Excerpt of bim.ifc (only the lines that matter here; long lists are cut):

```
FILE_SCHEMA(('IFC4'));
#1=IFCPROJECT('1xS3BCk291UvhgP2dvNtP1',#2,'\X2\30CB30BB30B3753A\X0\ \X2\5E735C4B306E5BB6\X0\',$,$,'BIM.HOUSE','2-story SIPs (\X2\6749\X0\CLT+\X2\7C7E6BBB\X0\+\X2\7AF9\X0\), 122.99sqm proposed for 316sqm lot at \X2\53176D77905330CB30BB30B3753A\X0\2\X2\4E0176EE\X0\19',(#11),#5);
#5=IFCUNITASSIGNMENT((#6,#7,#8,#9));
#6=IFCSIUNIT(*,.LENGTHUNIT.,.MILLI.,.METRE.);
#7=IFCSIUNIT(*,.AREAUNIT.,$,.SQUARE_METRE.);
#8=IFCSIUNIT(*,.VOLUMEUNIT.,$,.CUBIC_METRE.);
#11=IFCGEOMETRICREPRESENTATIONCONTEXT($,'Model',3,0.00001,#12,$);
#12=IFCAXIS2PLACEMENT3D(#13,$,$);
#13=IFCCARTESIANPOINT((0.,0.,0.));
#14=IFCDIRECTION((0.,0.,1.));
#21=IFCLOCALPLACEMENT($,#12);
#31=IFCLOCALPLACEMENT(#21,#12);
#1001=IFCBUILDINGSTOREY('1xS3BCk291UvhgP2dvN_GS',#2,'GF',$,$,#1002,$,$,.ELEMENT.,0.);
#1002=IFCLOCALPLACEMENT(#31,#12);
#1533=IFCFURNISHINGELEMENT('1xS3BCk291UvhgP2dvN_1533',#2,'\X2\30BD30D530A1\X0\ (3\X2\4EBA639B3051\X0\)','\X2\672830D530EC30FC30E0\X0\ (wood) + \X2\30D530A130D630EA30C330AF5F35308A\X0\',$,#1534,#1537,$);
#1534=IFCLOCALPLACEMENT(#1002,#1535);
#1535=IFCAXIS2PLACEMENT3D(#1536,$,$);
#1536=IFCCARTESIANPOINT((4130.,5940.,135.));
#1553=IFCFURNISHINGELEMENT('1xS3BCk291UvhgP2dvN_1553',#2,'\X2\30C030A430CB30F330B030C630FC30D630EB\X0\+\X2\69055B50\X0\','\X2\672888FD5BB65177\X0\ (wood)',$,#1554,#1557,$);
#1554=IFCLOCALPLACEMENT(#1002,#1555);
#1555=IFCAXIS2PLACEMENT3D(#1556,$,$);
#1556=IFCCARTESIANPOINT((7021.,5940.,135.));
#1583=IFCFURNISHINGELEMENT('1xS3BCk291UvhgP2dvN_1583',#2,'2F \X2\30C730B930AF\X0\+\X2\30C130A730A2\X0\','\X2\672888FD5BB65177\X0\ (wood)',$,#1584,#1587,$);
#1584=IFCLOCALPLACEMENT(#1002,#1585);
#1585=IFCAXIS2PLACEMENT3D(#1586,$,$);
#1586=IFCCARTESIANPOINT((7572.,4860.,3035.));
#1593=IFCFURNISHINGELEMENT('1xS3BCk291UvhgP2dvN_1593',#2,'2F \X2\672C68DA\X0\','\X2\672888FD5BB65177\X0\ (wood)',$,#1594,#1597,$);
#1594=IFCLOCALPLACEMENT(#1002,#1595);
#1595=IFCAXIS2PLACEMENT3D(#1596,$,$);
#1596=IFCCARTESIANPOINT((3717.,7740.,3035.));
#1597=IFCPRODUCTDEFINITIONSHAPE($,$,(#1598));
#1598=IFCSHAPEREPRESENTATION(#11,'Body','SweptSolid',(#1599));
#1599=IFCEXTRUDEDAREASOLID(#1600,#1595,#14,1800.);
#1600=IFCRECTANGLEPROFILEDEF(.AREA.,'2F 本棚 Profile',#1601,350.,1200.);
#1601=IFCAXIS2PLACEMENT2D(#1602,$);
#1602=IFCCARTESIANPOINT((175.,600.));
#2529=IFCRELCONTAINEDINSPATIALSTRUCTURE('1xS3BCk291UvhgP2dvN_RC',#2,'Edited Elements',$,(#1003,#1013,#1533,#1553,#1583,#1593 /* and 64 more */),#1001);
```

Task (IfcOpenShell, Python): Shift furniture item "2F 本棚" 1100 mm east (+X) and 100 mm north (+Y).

```python
import ifcopenshell
import ifcopenshell.api.geometry
import ifcopenshell.util.placement

model = ifcopenshell.open("bim.ifc")

item = model.by_guid("1xS3BCk291UvhgP2dvN_1593")
matrix = ifcopenshell.util.placement.get_local_placement(item.ObjectPlacement)
matrix[0, 3] += 1100.0
matrix[1, 3] += 100.0
ifcopenshell.api.geometry.edit_object_placement(model, product=item, matrix=matrix, is_si=False)

print(ifcopenshell.util.placement.get_local_placement(item.ObjectPlacement).round(3) + 0.0)

model.write("bim_v2.ifc")
```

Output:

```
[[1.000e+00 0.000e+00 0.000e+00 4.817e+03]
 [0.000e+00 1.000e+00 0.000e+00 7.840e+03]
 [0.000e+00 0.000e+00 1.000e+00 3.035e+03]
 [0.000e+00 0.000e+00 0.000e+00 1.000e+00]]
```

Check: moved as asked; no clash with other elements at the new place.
